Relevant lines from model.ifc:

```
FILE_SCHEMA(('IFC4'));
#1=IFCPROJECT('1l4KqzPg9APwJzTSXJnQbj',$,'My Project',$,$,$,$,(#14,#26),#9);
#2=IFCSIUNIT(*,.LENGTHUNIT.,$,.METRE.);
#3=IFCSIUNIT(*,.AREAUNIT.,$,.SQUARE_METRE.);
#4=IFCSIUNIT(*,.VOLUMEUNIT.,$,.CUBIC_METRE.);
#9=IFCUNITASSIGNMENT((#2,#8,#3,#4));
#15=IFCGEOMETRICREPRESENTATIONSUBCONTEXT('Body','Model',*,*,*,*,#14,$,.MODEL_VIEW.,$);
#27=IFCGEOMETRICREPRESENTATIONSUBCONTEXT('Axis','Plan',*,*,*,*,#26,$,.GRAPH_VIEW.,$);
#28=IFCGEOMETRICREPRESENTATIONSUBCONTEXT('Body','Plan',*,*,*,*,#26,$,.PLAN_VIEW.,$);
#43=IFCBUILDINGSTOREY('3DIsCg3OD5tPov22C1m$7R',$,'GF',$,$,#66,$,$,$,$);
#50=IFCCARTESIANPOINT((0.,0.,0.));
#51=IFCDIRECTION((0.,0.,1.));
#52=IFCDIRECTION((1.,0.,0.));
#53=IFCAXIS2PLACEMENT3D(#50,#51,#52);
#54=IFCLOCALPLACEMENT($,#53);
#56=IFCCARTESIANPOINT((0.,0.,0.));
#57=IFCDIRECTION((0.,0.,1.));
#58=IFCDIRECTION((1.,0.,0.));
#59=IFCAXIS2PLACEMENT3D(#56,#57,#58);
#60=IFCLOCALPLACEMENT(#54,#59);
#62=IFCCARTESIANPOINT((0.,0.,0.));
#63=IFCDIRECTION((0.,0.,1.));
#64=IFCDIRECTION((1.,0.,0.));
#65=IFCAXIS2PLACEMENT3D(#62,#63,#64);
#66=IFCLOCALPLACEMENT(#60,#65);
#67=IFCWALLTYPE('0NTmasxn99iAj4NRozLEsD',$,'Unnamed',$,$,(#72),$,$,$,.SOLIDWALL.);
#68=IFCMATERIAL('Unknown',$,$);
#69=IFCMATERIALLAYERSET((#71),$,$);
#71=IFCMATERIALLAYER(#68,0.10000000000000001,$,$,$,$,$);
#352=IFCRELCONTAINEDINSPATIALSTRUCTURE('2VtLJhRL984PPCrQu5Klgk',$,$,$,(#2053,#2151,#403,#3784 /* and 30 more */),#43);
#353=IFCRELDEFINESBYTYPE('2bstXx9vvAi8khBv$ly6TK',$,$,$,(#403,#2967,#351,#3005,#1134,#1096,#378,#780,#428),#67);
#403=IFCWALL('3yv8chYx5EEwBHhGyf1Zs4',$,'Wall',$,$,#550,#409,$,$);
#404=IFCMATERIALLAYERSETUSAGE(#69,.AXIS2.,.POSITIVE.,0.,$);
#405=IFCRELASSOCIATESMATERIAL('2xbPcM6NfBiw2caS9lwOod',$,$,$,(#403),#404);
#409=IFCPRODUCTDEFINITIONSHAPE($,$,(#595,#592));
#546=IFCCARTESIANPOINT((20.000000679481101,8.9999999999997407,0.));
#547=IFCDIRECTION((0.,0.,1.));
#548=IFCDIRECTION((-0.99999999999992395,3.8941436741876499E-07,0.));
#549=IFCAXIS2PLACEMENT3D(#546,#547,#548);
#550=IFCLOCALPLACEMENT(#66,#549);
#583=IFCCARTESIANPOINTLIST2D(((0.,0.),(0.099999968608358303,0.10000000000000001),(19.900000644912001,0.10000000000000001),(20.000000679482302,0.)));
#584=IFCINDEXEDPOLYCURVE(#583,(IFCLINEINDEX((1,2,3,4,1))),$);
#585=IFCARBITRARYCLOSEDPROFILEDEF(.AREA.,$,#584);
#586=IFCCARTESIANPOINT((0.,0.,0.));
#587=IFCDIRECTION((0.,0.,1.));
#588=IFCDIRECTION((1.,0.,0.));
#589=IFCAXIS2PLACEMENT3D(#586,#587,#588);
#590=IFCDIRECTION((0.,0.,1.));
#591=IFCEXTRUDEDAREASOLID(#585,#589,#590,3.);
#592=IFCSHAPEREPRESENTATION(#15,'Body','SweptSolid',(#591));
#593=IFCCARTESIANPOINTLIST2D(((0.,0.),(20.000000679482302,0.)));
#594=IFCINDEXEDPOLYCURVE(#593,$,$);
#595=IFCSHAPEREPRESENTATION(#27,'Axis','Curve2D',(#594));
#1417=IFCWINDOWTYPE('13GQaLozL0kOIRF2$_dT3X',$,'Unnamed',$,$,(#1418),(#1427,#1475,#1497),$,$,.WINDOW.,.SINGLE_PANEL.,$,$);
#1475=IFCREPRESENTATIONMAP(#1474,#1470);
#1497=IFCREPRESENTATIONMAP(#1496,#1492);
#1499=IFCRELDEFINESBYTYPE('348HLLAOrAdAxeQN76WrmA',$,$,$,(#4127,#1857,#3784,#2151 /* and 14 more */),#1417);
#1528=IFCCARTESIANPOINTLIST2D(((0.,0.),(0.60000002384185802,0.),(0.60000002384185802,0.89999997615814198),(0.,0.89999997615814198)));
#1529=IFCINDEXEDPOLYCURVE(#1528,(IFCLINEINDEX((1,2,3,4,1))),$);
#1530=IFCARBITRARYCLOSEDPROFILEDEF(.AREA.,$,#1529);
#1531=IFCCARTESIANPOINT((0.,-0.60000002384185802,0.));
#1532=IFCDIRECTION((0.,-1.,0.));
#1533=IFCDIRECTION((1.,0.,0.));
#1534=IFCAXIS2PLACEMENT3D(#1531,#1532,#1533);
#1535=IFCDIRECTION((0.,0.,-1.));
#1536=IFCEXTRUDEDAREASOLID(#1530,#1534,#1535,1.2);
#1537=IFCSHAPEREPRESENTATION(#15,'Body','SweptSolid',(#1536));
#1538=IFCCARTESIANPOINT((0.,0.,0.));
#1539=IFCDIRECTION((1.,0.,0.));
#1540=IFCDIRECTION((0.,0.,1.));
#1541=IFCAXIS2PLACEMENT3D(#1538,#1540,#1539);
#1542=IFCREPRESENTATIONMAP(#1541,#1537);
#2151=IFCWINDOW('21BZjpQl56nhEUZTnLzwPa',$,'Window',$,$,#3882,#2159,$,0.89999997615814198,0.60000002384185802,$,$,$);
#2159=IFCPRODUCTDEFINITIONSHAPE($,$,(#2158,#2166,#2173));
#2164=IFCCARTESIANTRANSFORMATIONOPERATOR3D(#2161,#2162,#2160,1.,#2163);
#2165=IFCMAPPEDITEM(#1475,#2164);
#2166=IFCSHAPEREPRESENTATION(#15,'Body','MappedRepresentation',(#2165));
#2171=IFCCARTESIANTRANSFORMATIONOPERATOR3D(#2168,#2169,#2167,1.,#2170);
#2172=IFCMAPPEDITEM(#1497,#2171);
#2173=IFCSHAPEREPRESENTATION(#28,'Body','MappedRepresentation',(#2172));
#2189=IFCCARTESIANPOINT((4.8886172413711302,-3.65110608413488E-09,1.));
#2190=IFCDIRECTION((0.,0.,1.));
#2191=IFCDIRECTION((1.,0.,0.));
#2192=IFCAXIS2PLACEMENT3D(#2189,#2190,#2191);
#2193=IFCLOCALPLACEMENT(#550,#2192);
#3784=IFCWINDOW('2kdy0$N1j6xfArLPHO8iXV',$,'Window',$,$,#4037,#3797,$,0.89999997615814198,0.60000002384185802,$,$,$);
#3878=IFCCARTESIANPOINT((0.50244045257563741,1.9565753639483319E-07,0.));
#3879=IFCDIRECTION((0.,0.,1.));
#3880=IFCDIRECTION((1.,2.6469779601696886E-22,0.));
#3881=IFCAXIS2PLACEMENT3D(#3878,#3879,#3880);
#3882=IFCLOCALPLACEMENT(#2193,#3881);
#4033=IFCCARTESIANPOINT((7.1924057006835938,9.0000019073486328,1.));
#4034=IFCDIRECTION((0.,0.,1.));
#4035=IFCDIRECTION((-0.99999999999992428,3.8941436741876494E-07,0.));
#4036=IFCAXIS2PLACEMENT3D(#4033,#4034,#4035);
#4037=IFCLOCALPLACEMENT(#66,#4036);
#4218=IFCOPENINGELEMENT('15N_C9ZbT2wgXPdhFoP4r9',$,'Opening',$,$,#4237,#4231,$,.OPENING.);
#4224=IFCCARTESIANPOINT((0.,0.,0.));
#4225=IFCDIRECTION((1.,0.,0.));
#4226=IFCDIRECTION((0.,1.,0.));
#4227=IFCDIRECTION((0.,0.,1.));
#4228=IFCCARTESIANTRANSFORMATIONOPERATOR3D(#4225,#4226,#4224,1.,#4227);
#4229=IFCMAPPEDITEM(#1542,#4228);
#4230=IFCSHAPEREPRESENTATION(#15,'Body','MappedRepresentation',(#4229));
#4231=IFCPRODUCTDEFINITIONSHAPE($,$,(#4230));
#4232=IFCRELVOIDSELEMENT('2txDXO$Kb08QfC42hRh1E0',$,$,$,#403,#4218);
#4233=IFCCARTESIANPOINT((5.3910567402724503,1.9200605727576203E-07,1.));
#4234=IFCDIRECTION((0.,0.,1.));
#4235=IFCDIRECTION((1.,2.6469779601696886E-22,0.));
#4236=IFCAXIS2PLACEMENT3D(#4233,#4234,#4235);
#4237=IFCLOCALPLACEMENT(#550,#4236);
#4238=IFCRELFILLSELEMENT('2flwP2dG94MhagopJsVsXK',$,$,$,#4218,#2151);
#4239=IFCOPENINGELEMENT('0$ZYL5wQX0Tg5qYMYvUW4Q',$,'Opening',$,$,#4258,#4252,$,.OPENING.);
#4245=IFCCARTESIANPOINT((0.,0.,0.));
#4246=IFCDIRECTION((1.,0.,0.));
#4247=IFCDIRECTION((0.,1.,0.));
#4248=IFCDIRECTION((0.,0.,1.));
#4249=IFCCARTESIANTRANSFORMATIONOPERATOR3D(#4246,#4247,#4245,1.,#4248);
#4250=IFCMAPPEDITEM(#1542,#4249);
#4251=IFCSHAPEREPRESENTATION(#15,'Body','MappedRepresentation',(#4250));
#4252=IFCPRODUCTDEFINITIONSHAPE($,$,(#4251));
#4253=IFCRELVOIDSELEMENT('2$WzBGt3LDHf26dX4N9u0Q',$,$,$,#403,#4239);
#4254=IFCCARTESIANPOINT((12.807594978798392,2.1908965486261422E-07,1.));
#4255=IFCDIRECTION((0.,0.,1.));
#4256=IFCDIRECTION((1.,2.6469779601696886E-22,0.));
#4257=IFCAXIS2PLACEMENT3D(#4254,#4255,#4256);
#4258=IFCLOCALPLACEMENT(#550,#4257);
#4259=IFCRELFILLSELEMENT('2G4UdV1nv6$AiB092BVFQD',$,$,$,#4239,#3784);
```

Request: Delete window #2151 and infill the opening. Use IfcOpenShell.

```python
import ifcopenshell
import ifcopenshell.api.feature
import ifcopenshell.api.root
import ifcopenshell.geom
import ifcopenshell.util.shape

model = ifcopenshell.open("model.ifc")
settings = ifcopenshell.geom.settings()


def volume(element):
    """Net volume in cubic metres, openings subtracted."""
    shape = ifcopenshell.geom.create_shape(settings, element)
    return ifcopenshell.util.shape.get_volume(shape.geometry)


window = model.by_guid("21BZjpQl56nhEUZTnLzwPa")
opening = window.FillsVoids[0].RelatingOpeningElement
wall = opening.VoidsElements[0].RelatingBuildingElement
before = volume(wall)

ifcopenshell.api.root.remove_product(model, product=window)
ifcopenshell.api.feature.remove_feature(model, feature=opening)

after = volume(wall)

print(f"wall volume {before:.3f} -> {after:.3f} m3")

model.write("model_v2.ifc")
```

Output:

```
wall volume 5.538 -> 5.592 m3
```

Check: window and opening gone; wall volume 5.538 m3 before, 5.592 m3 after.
